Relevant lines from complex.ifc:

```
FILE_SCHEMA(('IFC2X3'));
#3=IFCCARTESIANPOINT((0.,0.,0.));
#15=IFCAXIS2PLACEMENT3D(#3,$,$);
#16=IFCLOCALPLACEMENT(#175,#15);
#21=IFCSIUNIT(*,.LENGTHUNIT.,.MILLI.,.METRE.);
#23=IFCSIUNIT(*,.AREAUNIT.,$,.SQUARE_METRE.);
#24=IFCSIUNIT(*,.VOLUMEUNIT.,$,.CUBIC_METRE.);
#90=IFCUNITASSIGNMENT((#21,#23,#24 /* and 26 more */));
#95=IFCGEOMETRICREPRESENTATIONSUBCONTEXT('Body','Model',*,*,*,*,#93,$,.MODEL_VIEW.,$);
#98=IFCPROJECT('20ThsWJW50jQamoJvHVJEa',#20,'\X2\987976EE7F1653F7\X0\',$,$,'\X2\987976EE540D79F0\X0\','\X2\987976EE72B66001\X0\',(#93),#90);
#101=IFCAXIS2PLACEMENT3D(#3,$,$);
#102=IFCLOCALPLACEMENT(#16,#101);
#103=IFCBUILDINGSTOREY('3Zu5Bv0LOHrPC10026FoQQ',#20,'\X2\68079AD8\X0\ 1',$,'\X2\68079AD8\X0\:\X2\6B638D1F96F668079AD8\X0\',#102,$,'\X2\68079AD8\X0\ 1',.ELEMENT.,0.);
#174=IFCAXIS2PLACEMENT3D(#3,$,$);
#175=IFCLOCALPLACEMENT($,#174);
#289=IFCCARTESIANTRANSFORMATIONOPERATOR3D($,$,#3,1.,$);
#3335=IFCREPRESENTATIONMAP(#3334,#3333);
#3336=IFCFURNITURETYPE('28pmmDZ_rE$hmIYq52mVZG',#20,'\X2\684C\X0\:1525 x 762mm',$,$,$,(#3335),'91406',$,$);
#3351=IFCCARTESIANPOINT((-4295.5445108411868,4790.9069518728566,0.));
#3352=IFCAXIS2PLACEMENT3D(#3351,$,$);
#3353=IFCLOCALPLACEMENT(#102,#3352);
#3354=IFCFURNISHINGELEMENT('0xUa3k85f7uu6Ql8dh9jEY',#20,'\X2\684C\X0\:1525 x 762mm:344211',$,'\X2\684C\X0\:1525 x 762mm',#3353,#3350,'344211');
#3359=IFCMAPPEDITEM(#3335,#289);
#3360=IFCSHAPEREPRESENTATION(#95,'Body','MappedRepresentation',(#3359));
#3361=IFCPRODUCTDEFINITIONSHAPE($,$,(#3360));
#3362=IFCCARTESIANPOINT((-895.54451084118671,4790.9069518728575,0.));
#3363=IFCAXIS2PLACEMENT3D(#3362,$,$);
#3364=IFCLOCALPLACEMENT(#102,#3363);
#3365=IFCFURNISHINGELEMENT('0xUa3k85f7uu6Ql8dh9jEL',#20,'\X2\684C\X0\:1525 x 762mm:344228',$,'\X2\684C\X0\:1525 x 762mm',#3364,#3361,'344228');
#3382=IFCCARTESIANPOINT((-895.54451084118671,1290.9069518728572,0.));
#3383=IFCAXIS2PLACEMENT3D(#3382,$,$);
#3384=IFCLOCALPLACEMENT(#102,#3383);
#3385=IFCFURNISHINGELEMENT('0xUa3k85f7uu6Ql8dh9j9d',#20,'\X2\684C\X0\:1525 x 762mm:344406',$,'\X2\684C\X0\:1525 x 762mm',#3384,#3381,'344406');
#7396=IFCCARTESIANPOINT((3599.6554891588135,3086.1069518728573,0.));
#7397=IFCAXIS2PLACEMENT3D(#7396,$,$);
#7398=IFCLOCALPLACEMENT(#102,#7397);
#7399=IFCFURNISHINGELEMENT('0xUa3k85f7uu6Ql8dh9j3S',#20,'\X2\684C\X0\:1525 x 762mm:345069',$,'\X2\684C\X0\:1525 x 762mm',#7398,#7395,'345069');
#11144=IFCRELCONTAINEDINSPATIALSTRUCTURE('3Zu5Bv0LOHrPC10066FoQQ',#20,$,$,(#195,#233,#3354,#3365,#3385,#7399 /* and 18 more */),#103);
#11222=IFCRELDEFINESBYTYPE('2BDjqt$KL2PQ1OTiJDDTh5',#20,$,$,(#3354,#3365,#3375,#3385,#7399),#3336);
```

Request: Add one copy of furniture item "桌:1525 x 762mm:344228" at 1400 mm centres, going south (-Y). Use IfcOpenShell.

```python
import numpy as np
import ifcopenshell
import ifcopenshell.api.geometry
import ifcopenshell.api.root
import ifcopenshell.util.element
import ifcopenshell.util.placement

model = ifcopenshell.open("complex.ifc")


def reuse_history(source, copy):
    """copy_class also copies each property set's owner history, people and application; keep the originals."""
    for rel in copy.IsDefinedBy:
        if rel.is_a("IfcRelDefinesByProperties") and (history := rel.RelatingPropertyDefinition.OwnerHistory):
            rel.RelatingPropertyDefinition.OwnerHistory = source.OwnerHistory
            ifcopenshell.util.element.remove_deep2(model, history)


source = model.by_guid("0xUa3k85f7uu6Ql8dh9jEL")
base = ifcopenshell.util.placement.get_local_placement(source.ObjectPlacement)
step = np.array([0.0, -1.0, 0.0]) * 1400.0

for i in range(1, 2):
    copy = ifcopenshell.api.root.copy_class(model, product=source)
    copy.Representation = ifcopenshell.util.element.copy_deep(
        model, source.Representation, exclude=["IfcGeometricRepresentationContext", "IfcRepresentationMap"]
    )
    copy.Name = "桌:1525 x 762mm"
    copy.Tag = None
    reuse_history(source, copy)
    matrix = base.copy()
    matrix[:3, 3] += i * step
    print("added at", matrix[:3, 3].round(3) + 0.0)
    ifcopenshell.api.geometry.edit_object_placement(model, product=copy, matrix=matrix, is_si=False)

model.write("complex_edited.ifc")
```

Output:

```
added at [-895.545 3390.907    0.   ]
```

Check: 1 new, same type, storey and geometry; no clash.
